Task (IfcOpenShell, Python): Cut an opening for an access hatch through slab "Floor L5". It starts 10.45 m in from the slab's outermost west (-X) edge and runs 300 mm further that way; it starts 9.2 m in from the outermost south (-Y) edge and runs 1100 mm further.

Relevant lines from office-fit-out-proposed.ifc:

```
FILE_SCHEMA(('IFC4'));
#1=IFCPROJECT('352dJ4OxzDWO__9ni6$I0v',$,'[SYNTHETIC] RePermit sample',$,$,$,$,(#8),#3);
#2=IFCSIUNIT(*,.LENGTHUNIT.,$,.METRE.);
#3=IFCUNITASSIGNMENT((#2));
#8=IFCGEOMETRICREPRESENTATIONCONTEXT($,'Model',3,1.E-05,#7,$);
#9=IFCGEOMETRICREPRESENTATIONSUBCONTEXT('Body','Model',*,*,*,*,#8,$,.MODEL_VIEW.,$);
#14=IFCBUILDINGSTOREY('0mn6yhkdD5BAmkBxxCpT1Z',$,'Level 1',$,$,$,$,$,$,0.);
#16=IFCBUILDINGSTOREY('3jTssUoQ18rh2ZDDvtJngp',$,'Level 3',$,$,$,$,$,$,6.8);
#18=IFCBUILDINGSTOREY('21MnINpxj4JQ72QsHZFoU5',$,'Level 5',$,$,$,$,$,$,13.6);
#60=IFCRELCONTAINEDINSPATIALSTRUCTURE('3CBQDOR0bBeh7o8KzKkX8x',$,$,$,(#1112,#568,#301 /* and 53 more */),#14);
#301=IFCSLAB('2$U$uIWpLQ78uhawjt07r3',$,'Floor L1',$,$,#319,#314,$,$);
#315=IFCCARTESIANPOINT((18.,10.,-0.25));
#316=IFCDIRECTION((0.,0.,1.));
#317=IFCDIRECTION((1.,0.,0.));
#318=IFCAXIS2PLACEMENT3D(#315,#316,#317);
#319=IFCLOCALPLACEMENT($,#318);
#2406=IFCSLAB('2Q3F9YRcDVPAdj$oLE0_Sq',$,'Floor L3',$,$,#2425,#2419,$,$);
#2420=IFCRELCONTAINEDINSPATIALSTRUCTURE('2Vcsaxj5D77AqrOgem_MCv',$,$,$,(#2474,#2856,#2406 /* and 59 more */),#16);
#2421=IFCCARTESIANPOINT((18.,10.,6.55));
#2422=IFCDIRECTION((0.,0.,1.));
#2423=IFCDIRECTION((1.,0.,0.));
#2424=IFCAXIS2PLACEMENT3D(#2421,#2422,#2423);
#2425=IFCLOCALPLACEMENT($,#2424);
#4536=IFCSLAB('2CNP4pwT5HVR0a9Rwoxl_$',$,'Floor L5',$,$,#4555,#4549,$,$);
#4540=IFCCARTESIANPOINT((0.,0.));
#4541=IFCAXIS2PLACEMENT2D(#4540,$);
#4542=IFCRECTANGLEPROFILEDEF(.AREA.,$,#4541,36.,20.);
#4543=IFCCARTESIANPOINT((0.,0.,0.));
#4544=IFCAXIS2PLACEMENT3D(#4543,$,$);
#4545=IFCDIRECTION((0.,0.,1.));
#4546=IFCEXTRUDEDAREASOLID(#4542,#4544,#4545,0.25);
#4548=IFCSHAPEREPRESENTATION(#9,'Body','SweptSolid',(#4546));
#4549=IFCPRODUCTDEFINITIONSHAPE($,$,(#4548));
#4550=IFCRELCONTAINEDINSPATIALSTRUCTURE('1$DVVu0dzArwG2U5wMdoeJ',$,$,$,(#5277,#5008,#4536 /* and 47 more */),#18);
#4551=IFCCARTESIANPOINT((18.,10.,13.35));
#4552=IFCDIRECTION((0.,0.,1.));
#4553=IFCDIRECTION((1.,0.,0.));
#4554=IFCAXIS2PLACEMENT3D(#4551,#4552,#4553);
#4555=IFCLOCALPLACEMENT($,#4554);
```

```python
import numpy as np
import ifcopenshell
import ifcopenshell.api.feature
import ifcopenshell.api.geometry
import ifcopenshell.api.root
import ifcopenshell.geom
import ifcopenshell.util.placement
import ifcopenshell.util.representation
import ifcopenshell.util.shape
import ifcopenshell.util.unit

model = ifcopenshell.open("office-fit-out-proposed.ifc")
unit_scale = ifcopenshell.util.unit.calculate_unit_scale(model)
settings = ifcopenshell.geom.settings()


def volume(element):
    """Net volume in cubic metres, openings subtracted."""
    shape = ifcopenshell.geom.create_shape(settings, element)
    return ifcopenshell.util.shape.get_volume(shape.geometry)


slab = model.by_guid("2CNP4pwT5HVR0a9Rwoxl_$")
before = volume(slab)

# Extent in the slab's own axes, in metres. The edges named are its -X and -Y sides.
slab_shape = ifcopenshell.geom.create_shape(settings, slab)
vertices = ifcopenshell.util.shape.get_vertices(slab_shape.geometry)
x_min, y_min, bottom = vertices.min(axis=0)
top = vertices[:, 2].max()

opening = ifcopenshell.api.root.create_entity(model, ifc_class="IfcOpeningElement", name="Access hatch opening", predefined_type="OPENING")
context = ifcopenshell.util.representation.get_context(model, "Model", "Body", "MODEL_VIEW")
width, depth = 0.3, 1.1
outline = [(0.0, 0.0), (width, 0.0), (width, depth), (0.0, depth), (0.0, 0.0)]
# Overshoot both faces by 50 mm so the cut is clean.
shape = ifcopenshell.api.geometry.add_slab_representation(
    model, context=context, depth=top - bottom + 0.1, polyline=outline
)
ifcopenshell.api.geometry.assign_representation(model, product=opening, representation=shape)

matrix = ifcopenshell.util.placement.get_local_placement(slab.ObjectPlacement)
matrix[:, 3] = matrix @ np.append(np.array([x_min + 10.45, y_min + 9.2, bottom - 0.05]) / unit_scale, 1.0)
ifcopenshell.api.geometry.edit_object_placement(model, product=opening, matrix=matrix, is_si=False)
ifcopenshell.api.feature.add_feature(model, feature=opening, element=slab)

after = volume(slab)

print(f"slab volume {before:.3f} -> {after:.3f} m3")

model.write("office-fit-out-proposed-out.ifc")
```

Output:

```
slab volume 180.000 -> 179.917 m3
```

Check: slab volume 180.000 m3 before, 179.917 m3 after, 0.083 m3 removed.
